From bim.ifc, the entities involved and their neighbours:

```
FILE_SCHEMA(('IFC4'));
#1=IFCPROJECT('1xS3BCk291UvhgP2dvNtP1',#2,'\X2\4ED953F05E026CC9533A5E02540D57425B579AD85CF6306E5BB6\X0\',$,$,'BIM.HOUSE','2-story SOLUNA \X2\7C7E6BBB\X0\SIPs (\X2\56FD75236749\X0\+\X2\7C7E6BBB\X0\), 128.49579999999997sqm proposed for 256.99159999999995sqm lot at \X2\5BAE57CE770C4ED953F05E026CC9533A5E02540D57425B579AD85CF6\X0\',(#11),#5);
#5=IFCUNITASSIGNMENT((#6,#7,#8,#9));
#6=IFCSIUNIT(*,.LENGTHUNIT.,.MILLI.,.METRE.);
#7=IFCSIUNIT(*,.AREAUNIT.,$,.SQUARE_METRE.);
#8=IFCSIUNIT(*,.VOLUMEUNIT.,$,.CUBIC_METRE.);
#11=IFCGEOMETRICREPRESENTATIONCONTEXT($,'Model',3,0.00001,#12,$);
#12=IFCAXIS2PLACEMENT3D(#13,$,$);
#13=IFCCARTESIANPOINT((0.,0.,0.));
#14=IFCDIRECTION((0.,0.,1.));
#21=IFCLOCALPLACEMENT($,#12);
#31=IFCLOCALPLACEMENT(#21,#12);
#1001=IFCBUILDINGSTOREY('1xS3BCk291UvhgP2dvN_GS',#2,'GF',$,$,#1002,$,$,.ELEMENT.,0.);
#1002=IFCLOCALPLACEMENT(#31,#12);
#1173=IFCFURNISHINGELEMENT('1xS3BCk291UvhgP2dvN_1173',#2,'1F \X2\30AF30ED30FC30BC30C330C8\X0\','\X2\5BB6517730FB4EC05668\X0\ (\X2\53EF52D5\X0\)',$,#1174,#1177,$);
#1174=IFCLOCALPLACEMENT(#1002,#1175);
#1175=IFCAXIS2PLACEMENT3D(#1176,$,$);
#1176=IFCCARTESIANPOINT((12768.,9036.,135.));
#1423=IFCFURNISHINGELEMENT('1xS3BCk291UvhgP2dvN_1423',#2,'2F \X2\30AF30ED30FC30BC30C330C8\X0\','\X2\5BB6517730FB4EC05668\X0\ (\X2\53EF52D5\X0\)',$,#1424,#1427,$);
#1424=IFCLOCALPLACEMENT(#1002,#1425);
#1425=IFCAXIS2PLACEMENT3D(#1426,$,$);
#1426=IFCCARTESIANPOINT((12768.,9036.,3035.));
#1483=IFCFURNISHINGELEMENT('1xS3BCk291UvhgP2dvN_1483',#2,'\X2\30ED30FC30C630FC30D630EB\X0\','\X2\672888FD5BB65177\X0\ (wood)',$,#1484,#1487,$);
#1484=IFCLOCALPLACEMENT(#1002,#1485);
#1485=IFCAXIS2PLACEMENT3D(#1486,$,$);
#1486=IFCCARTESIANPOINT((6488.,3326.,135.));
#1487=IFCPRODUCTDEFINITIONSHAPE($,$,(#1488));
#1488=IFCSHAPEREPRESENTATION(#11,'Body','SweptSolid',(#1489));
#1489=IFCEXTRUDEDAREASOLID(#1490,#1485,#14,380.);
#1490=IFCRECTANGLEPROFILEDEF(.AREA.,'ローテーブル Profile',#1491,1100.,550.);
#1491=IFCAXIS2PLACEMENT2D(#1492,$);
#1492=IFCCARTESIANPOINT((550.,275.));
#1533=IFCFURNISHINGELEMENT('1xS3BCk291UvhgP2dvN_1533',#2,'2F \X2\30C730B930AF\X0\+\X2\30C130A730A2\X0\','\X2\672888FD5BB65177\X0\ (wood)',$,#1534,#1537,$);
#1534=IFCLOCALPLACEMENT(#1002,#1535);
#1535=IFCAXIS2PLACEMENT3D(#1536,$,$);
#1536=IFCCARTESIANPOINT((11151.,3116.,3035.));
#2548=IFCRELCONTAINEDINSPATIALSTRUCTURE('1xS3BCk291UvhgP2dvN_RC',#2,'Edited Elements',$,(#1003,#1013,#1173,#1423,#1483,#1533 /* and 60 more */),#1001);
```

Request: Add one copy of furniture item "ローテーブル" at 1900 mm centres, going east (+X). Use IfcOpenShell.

```python
import numpy as np
import ifcopenshell
import ifcopenshell.api.geometry
import ifcopenshell.api.root
import ifcopenshell.util.element
import ifcopenshell.util.placement
import ifcopenshell.util.unit

model = ifcopenshell.open("bim.ifc")
unit_scale = ifcopenshell.util.unit.calculate_unit_scale(model)


def reuse_history(source, copy):
    """copy_class also copies each property set's owner history, people and application; keep the originals."""
    for rel in copy.IsDefinedBy:
        if rel.is_a("IfcRelDefinesByProperties") and (history := rel.RelatingPropertyDefinition.OwnerHistory):
            rel.RelatingPropertyDefinition.OwnerHistory = source.OwnerHistory
            ifcopenshell.util.element.remove_deep2(model, history)


source = model.by_guid("1xS3BCk291UvhgP2dvN_1483")
base = ifcopenshell.util.placement.get_local_placement(source.ObjectPlacement)
step = np.array([1.0, 0.0, 0.0]) * 1.9 / unit_scale

for i in range(1, 2):
    copy = ifcopenshell.api.root.copy_class(model, product=source)
    copy.Representation = ifcopenshell.util.element.copy_deep(
        model, source.Representation, exclude=["IfcGeometricRepresentationContext", "IfcRepresentationMap"]
    )
    reuse_history(source, copy)
    matrix = base.copy()
    matrix[:3, 3] += i * step
    print("added at", matrix[:3, 3].round(3) + 0.0)
    ifcopenshell.api.geometry.edit_object_placement(model, product=copy, matrix=matrix, is_si=False)

model.write("bim_updated.ifc")
```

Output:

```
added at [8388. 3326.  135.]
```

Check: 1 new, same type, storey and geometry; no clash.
